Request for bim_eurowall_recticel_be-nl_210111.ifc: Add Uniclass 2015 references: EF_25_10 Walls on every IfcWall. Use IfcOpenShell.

First a look at what the model holds.

```python
import ifcopenshell

model = ifcopenshell.open("bim_eurowall_recticel_be-nl_210111.ifc")
print(model.schema)
print("classifications:", [c.Name for c in model.by_type("IfcClassification")])
for ifc_class in ("IfcDoor", "IfcRoof", "IfcStair", "IfcWall", "IfcWindow"):
    print(ifc_class, len(model.by_type(ifc_class)))
```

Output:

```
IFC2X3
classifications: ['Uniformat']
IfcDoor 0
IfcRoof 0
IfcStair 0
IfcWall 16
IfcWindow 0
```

```python
import ifcopenshell
import ifcopenshell.api.classification

model = ifcopenshell.open("bim_eurowall_recticel_be-nl_210111.ifc")

# IFC2X3 requires Source and Edition and has no link from the project to the system.
system = model.create_entity("IfcClassification", Source="NBS", Edition="2015", Name="Uniclass 2015")

codes = {
    "IfcWall": ("EF_25_10", "Walls"),
}
for ifc_class, (code, name) in codes.items():
    products = model.by_type(ifc_class)
    ifcopenshell.api.classification.add_reference(
        model, products=products, classification=system, identification=code, name=name
    )
    print(code, len(products))

model.write("bim_eurowall_recticel_be-nl_210111_edited.ifc")
```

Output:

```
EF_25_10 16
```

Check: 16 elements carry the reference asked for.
